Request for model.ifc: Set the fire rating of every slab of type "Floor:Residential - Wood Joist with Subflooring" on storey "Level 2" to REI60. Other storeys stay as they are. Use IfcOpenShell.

First a look at what the model holds.

```python
import ifcopenshell
import ifcopenshell.util.element

model = ifcopenshell.open("model.ifc")
print(model.schema)
storey = next(s for s in model.by_type("IfcBuildingStorey") if s.Name == "Level 2")
slabs = [e for e in ifcopenshell.util.element.get_decomposition(storey) if e.is_a("IfcSlab")]
seen = {}
for e in slabs:
    element_type = ifcopenshell.util.element.get_type(e)
    key = (element_type.Name if element_type != e and element_type else None, ifcopenshell.util.element.get_pset(e, "Pset_SlabCommon", "FireRating"))
    seen[key] = seen.get(key, 0) + 1
for (name, value), count in sorted(seen.items(), key=str):
    print(count, "x", name, "|", value)
```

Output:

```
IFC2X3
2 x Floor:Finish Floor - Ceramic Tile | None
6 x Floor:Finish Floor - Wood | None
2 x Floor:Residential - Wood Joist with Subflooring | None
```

```python
import ifcopenshell
import ifcopenshell.api.pset
import ifcopenshell.util.element

model = ifcopenshell.open("model.ifc")

storey = next(s for s in model.by_type("IfcBuildingStorey") if s.Name == "Level 2")
slabs = [e for e in ifcopenshell.util.element.get_decomposition(storey) if e.is_a("IfcSlab")]

count = 0
for e in slabs:
    element_type = ifcopenshell.util.element.get_type(e)
    if element_type in (None, e) or element_type.Name != "Floor:Residential - Wood Joist with Subflooring":
        continue
    # add_pset returns the element's existing set when there is one.
    pset = ifcopenshell.api.pset.add_pset(model, product=e, name="Pset_SlabCommon")
    ifcopenshell.api.pset.edit_pset(model, pset=pset, properties={"FireRating": "REI60"})
    count += 1

print(count, "slabs updated")

model.write("model_updated.ifc")
```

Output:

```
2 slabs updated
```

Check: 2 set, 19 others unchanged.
